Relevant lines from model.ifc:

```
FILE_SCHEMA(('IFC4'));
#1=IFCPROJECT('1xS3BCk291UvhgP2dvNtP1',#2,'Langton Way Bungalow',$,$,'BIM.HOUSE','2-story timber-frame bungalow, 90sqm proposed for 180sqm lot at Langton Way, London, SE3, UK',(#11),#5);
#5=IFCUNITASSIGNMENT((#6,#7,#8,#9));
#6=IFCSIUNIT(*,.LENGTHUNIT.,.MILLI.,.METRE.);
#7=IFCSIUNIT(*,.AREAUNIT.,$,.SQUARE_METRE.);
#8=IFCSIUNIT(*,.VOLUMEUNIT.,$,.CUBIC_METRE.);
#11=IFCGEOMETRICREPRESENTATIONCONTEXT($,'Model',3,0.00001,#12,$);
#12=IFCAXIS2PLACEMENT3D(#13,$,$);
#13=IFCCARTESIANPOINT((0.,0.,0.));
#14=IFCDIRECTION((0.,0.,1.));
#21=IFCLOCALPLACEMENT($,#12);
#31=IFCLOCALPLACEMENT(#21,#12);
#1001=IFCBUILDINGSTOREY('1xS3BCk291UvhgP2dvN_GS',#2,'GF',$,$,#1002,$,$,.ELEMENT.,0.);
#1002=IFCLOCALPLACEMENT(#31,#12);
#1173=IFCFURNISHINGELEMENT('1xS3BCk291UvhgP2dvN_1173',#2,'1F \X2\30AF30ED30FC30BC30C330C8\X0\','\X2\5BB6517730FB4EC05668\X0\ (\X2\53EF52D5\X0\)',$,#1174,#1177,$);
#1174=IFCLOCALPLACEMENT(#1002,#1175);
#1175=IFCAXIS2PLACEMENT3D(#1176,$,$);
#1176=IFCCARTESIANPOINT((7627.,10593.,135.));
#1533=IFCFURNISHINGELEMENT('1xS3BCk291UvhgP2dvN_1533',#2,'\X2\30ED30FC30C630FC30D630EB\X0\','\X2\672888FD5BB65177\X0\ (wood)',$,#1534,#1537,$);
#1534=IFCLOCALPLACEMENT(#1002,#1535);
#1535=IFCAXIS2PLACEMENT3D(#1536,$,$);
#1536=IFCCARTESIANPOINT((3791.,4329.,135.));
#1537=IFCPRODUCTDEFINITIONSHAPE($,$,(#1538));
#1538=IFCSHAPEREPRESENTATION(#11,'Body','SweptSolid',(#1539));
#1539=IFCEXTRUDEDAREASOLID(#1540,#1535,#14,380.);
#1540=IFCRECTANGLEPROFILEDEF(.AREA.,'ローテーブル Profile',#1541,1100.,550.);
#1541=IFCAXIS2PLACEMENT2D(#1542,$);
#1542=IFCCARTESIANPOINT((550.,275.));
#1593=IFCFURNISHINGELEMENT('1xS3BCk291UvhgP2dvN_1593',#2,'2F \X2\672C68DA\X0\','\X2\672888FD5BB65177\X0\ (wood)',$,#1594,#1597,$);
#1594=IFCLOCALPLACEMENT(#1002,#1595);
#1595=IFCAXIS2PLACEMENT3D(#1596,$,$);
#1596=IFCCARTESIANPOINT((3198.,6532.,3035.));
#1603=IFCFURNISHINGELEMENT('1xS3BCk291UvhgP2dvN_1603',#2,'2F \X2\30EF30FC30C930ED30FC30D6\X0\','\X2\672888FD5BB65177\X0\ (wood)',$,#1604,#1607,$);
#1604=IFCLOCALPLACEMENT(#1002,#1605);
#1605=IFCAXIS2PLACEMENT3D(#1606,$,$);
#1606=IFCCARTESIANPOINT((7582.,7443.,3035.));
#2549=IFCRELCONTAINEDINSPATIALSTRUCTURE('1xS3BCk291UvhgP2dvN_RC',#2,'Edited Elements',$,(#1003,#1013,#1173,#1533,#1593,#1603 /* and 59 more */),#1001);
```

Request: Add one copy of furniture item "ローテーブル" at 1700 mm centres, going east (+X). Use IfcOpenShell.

```python
import numpy as np
import ifcopenshell
import ifcopenshell.api.geometry
import ifcopenshell.api.root
import ifcopenshell.util.element
import ifcopenshell.util.placement
import ifcopenshell.util.unit

model = ifcopenshell.open("model.ifc")
unit_scale = ifcopenshell.util.unit.calculate_unit_scale(model)


def reuse_history(source, copy):
    """copy_class also copies each property set's owner history, people and application; keep the originals."""
    for rel in copy.IsDefinedBy:
        if rel.is_a("IfcRelDefinesByProperties") and (history := rel.RelatingPropertyDefinition.OwnerHistory):
            rel.RelatingPropertyDefinition.OwnerHistory = source.OwnerHistory
            ifcopenshell.util.element.remove_deep2(model, history)


source = model.by_guid("1xS3BCk291UvhgP2dvN_1533")
base = ifcopenshell.util.placement.get_local_placement(source.ObjectPlacement)
step = np.array([1.0, 0.0, 0.0]) * 1.7 / unit_scale

for i in range(1, 2):
    copy = ifcopenshell.api.root.copy_class(model, product=source)
    copy.Representation = ifcopenshell.util.element.copy_deep(
        model, source.Representation, exclude=["IfcGeometricRepresentationContext", "IfcRepresentationMap"]
    )
    reuse_history(source, copy)
    matrix = base.copy()
    matrix[:3, 3] += i * step
    print("added at", matrix[:3, 3].round(3) + 0.0)
    ifcopenshell.api.geometry.edit_object_placement(model, product=copy, matrix=matrix, is_si=False)

model.write("model_updated.ifc")
```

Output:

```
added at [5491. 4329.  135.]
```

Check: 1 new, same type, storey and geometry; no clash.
